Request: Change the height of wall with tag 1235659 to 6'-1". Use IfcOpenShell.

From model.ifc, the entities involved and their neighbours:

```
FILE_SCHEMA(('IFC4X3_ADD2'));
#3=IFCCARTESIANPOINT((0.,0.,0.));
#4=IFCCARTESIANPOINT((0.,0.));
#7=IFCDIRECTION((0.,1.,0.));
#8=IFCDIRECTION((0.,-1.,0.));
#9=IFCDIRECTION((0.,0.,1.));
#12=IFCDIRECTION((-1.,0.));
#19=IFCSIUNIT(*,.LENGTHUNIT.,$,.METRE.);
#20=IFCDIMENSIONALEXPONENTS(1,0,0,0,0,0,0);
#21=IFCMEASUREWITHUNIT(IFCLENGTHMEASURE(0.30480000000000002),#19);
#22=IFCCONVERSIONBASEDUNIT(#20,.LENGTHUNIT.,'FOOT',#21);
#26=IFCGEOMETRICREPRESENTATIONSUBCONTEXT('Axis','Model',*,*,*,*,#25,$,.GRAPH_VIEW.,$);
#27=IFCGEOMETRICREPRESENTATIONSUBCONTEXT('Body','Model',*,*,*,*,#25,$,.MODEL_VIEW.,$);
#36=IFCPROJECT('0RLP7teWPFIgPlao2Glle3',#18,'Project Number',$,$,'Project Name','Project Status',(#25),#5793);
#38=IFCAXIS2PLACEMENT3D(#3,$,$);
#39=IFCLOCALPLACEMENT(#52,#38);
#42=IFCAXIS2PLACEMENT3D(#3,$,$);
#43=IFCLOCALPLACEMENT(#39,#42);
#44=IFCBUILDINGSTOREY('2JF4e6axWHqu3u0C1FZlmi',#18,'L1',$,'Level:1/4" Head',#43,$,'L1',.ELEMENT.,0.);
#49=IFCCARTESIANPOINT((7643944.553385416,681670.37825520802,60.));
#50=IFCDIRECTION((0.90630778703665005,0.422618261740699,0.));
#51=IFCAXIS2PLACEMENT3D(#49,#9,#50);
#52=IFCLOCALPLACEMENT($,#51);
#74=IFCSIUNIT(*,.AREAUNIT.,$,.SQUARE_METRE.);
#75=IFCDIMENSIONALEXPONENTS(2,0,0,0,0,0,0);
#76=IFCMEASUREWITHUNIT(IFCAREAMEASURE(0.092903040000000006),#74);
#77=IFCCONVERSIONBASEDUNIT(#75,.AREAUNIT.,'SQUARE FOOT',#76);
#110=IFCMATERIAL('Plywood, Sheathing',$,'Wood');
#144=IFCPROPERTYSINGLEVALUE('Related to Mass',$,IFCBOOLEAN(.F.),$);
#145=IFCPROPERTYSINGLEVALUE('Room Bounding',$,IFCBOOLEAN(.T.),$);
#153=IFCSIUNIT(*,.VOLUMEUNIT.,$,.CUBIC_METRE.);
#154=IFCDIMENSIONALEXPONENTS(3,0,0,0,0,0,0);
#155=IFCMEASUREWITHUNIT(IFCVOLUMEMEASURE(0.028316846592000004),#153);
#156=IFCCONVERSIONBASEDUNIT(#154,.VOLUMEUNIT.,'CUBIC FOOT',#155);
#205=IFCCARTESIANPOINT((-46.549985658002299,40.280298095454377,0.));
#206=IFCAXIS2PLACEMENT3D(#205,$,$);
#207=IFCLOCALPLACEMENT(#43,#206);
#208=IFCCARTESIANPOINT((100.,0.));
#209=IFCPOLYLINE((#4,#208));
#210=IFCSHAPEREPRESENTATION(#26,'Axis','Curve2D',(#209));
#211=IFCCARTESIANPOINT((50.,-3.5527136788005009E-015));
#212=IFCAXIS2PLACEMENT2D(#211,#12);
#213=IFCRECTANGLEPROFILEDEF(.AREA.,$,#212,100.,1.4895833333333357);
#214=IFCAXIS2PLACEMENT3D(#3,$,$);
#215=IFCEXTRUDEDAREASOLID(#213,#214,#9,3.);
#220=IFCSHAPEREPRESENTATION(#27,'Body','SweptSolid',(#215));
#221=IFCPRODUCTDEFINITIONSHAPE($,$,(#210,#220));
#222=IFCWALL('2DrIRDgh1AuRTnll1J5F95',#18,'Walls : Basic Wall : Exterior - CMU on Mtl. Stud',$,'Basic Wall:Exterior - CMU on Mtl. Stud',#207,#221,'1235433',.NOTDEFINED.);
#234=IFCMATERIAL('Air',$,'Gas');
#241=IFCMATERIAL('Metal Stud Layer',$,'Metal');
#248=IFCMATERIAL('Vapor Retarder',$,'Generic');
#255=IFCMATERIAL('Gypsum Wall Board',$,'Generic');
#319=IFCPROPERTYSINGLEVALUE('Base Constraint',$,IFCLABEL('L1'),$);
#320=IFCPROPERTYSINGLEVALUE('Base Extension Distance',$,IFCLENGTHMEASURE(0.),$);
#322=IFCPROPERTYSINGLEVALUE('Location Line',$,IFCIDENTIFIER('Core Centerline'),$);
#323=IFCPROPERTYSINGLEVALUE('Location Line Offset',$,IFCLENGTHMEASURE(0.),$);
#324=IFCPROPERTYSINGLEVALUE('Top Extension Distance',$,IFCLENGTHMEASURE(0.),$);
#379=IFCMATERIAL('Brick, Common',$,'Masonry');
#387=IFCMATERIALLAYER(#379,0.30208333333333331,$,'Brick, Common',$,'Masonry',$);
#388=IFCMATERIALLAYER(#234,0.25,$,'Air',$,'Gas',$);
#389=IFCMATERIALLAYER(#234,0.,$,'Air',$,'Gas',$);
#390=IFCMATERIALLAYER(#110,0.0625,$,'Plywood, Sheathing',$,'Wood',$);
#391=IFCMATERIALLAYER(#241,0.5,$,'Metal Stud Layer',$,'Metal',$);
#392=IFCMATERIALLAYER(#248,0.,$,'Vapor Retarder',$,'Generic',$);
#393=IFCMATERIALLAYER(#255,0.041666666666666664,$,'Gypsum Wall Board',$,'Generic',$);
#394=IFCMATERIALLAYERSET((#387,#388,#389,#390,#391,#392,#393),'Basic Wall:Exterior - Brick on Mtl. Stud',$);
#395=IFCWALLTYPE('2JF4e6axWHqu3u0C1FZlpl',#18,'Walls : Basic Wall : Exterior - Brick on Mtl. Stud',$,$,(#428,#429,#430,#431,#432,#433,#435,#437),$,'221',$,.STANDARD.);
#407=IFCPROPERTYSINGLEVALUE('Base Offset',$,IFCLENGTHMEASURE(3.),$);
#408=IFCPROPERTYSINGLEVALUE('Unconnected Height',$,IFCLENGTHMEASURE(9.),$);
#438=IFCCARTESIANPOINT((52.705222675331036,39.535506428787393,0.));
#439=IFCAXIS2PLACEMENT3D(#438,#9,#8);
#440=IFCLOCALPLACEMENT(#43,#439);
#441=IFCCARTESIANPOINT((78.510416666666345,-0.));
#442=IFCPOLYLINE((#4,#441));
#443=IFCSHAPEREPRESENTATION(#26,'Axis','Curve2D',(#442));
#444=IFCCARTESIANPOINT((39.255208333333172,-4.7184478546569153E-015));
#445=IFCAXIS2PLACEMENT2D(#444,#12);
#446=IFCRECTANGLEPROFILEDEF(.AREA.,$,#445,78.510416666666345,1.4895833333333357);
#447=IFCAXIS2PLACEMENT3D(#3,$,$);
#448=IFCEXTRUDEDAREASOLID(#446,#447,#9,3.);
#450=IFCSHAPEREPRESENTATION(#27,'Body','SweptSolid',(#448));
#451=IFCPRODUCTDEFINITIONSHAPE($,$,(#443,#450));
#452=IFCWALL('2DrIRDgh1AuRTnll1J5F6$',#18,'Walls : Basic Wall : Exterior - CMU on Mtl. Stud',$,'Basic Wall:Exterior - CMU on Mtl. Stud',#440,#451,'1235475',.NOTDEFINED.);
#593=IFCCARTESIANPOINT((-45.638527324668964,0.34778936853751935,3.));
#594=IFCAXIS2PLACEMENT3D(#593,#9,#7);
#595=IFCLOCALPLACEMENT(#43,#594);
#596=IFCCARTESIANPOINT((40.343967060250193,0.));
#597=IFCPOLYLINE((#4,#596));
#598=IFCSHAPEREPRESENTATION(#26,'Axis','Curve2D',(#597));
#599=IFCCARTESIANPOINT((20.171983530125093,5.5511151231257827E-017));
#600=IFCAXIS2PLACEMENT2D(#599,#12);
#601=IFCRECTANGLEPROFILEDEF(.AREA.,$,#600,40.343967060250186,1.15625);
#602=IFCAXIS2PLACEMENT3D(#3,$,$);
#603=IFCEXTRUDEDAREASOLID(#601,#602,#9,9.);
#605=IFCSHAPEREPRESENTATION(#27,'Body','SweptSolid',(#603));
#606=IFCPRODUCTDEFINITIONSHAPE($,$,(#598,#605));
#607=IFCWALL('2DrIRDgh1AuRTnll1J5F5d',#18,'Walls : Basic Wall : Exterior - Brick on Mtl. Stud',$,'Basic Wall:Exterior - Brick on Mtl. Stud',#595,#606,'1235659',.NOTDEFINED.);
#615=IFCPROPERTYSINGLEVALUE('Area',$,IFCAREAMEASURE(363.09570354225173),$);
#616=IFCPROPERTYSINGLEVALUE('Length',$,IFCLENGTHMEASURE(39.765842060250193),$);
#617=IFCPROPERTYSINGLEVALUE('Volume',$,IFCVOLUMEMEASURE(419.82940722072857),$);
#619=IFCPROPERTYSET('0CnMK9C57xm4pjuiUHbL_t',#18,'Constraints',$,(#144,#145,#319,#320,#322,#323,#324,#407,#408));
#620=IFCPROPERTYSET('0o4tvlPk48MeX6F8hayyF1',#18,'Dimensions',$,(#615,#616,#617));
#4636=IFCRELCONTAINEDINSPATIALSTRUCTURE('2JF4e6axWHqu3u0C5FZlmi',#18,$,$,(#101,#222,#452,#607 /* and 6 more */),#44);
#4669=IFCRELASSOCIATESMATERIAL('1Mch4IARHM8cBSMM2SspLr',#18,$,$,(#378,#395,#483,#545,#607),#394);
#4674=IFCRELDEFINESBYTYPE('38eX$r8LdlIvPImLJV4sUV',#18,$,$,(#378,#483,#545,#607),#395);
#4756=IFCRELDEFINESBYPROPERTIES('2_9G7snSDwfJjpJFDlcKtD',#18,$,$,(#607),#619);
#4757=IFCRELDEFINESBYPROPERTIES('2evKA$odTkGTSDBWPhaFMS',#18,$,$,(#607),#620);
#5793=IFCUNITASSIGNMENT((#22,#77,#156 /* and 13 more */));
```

```python
import ifcopenshell
import ifcopenshell.api.pset
import ifcopenshell.geom
import ifcopenshell.util.element
import ifcopenshell.util.representation
import ifcopenshell.util.shape
import ifcopenshell.util.unit

model = ifcopenshell.open("model.ifc")
unit_scale = ifcopenshell.util.unit.calculate_unit_scale(model)
area_scale = ifcopenshell.util.unit.calculate_unit_scale(model, "AREAUNIT")
volume_scale = ifcopenshell.util.unit.calculate_unit_scale(model, "VOLUMEUNIT")
settings = ifcopenshell.geom.settings()


def volume(element):
    """Net volume in cubic metres, openings subtracted."""
    shape = ifcopenshell.geom.create_shape(settings, element)
    return ifcopenshell.util.shape.get_volume(shape.geometry)


wall = model.by_guid("2DrIRDgh1AuRTnll1J5F5d")
before = volume(wall)

body = ifcopenshell.util.representation.get_representation(wall, "Model", "Body")
solid = body.Items[0]
old_height = solid.Depth
solid.Depth = 73 * 0.0254 / unit_scale
after = volume(wall)
thickness = 0.3524  # wall thickness in metres

# Update the stored height, areas and volumes.
pset = model.by_id(ifcopenshell.util.element.get_pset(wall, "Constraints", should_inherit=False)["id"])
ifcopenshell.api.pset.edit_pset(model, pset=pset, properties={
    "Unconnected Height": model.create_entity("IfcLengthMeasure", solid.Depth),
})
pset = model.by_id(ifcopenshell.util.element.get_pset(wall, "Dimensions", should_inherit=False)["id"])
ifcopenshell.api.pset.edit_pset(model, pset=pset, properties={
    "Area": model.create_entity("IfcAreaMeasure", after / thickness / area_scale),
    "Volume": model.create_entity("IfcVolumeMeasure", after / volume_scale),
})

print(f"height {old_height:g} -> {solid.Depth:g}, volume {before:.3f} -> {after:.3f} m3")

model.write("model_edited.ifc")
```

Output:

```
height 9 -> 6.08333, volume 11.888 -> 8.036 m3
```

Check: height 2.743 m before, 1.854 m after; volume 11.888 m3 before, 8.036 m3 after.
